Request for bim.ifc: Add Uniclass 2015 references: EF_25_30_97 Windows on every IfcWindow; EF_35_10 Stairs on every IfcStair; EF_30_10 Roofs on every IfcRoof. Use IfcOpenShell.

First a look at what the model holds.

```python
import ifcopenshell

model = ifcopenshell.open("bim.ifc")
print(model.schema)
print("classifications:", [c.Name for c in model.by_type("IfcClassification")])
for ifc_class in ("IfcDoor", "IfcRoof", "IfcStair", "IfcWall", "IfcWindow"):
    print(ifc_class, len(model.by_type(ifc_class)))
```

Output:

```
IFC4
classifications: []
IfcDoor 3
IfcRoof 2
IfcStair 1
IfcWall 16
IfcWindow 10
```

```python
import ifcopenshell
import ifcopenshell.api.classification

model = ifcopenshell.open("bim.ifc")

system = ifcopenshell.api.classification.add_classification(model, classification="Uniclass 2015")

codes = {
    "IfcWindow": ("EF_25_30_97", "Windows"),
    "IfcStair": ("EF_35_10", "Stairs"),
    "IfcRoof": ("EF_30_10", "Roofs"),
}
for ifc_class, (code, name) in codes.items():
    products = model.by_type(ifc_class)
    ifcopenshell.api.classification.add_reference(
        model, products=products, classification=system, identification=code, name=name
    )
    print(code, len(products))

model.write("bim_v2.ifc")
```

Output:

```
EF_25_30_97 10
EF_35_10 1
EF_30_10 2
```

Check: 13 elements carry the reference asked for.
